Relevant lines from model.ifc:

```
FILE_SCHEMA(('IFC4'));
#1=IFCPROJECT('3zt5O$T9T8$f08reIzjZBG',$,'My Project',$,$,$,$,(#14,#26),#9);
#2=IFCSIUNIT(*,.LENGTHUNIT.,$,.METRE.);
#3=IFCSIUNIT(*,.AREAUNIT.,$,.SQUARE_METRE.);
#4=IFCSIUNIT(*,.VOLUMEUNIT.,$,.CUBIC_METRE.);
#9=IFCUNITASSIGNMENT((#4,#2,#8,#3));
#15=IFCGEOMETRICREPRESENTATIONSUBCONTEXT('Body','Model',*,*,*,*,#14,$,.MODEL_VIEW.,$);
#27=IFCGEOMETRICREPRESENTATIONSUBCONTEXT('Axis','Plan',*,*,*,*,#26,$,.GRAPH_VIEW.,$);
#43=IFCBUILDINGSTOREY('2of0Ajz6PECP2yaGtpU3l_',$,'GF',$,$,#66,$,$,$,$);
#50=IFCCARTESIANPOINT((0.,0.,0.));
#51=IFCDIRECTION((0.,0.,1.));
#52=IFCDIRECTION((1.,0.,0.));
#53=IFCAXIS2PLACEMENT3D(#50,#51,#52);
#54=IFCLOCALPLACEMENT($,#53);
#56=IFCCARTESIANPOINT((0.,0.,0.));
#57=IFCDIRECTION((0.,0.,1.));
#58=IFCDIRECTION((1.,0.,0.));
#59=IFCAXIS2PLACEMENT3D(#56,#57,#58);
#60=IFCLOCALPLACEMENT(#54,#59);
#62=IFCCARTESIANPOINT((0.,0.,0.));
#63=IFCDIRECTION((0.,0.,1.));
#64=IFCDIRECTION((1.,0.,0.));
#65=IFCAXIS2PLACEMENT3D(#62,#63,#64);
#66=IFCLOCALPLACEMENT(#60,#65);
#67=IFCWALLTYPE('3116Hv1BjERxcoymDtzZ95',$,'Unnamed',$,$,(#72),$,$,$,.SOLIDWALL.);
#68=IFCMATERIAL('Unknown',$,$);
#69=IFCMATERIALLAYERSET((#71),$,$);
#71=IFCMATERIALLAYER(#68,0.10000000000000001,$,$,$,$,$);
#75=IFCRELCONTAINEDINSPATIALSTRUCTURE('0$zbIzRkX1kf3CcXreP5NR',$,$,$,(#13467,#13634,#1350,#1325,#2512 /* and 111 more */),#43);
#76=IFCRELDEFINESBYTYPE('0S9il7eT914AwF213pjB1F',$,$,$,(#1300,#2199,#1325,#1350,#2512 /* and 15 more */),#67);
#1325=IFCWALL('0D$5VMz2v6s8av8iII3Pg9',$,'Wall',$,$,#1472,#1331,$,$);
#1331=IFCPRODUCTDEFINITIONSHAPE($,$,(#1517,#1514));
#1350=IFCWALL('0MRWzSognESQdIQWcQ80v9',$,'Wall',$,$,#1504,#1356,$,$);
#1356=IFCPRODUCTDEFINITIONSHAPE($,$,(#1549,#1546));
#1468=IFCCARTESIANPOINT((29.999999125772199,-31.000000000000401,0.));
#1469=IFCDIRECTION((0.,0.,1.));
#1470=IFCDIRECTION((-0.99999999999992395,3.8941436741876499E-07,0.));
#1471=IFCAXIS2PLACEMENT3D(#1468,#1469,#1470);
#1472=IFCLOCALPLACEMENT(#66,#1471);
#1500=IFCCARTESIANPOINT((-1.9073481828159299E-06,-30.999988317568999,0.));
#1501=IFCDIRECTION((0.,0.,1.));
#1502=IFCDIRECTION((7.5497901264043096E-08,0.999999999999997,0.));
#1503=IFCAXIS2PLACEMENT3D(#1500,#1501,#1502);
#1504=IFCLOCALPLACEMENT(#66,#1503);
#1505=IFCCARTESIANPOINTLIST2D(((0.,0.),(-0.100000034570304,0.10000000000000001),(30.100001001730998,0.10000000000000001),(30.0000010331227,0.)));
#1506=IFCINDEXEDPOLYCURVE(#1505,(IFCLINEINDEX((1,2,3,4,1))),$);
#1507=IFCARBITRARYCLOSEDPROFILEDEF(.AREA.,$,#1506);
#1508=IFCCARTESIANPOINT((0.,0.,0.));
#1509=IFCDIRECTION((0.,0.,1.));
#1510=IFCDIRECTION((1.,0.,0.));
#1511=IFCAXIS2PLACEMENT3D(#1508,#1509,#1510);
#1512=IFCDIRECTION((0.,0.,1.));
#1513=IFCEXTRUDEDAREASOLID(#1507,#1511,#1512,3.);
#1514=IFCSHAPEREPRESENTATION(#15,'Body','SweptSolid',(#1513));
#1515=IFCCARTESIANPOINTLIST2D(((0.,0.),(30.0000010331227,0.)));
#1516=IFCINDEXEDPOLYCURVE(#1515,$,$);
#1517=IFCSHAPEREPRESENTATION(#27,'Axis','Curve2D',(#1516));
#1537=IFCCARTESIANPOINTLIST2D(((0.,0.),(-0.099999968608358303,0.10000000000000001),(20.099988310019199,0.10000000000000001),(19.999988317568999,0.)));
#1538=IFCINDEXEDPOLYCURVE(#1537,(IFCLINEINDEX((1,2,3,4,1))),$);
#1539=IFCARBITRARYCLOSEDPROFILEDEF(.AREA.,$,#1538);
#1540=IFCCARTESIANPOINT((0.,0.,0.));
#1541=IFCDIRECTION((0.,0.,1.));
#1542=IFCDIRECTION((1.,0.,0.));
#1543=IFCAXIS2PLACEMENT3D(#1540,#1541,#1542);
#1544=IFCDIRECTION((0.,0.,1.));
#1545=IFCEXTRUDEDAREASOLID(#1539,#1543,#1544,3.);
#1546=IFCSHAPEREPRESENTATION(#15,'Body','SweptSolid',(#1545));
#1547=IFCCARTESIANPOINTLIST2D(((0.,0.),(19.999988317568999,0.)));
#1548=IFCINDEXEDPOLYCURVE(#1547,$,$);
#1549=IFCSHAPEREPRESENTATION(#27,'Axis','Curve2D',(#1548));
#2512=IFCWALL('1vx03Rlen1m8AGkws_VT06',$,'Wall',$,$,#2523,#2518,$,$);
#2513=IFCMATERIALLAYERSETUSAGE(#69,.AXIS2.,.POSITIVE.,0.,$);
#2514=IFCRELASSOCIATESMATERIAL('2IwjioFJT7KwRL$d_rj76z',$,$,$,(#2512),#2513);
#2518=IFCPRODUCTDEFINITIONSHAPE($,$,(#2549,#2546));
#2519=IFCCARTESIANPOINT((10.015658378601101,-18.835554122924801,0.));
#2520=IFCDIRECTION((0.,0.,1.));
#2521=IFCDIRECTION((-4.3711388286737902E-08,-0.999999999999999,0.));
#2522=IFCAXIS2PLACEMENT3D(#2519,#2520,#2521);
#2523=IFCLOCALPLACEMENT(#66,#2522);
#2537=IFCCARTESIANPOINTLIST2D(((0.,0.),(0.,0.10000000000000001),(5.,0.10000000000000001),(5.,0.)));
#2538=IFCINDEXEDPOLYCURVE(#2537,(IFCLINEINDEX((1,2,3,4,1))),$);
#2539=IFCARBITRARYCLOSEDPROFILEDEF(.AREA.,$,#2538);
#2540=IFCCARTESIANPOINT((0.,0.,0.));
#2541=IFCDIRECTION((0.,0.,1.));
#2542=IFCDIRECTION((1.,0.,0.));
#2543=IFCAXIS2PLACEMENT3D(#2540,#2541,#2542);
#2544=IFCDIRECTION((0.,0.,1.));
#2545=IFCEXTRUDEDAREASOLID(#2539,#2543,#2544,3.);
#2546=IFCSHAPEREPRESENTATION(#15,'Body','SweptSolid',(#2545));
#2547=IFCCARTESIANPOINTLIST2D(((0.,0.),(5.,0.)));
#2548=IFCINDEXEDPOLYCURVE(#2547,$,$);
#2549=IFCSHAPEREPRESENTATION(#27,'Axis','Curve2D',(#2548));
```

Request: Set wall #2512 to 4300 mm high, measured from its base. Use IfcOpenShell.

```python
import ifcopenshell
import ifcopenshell.geom
import ifcopenshell.util.representation
import ifcopenshell.util.shape

model = ifcopenshell.open("model.ifc")
settings = ifcopenshell.geom.settings()


def volume(element):
    """Net volume in cubic metres, openings subtracted."""
    shape = ifcopenshell.geom.create_shape(settings, element)
    return ifcopenshell.util.shape.get_volume(shape.geometry)


wall = model.by_id(2512)
before = volume(wall)

body = ifcopenshell.util.representation.get_representation(wall, "Model", "Body")
solid = body.Items[0]
old_height = solid.Depth
solid.Depth = 4.3
after = volume(wall)

print(f"height {old_height:g} -> {solid.Depth:g}, volume {before:.3f} -> {after:.3f} m3")

model.write("model-out.ifc")
```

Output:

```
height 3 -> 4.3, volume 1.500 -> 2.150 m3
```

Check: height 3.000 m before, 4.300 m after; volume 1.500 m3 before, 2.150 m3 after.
